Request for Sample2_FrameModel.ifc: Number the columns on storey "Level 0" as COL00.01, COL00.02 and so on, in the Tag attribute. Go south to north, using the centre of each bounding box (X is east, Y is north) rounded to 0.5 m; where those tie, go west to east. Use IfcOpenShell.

First a look at what the model holds.

```python
import ifcopenshell
import ifcopenshell.util.element
import ifcopenshell.util.placement

model = ifcopenshell.open("Sample2_FrameModel.ifc")
print(model.schema)
storey = next(s for s in model.by_type("IfcBuildingStorey") if s.Name == "Level 0")
columns = [e for e in ifcopenshell.util.element.get_decomposition(storey) if e.is_a("IfcColumn")]
for e in sorted(columns, key=lambda e: e.id()):
    origin = ifcopenshell.util.placement.get_local_placement(e.ObjectPlacement)[:3, 3]
    print(e.id(), e.Tag, e.Name, origin.round(2) + 0.0, sep=" | ")
```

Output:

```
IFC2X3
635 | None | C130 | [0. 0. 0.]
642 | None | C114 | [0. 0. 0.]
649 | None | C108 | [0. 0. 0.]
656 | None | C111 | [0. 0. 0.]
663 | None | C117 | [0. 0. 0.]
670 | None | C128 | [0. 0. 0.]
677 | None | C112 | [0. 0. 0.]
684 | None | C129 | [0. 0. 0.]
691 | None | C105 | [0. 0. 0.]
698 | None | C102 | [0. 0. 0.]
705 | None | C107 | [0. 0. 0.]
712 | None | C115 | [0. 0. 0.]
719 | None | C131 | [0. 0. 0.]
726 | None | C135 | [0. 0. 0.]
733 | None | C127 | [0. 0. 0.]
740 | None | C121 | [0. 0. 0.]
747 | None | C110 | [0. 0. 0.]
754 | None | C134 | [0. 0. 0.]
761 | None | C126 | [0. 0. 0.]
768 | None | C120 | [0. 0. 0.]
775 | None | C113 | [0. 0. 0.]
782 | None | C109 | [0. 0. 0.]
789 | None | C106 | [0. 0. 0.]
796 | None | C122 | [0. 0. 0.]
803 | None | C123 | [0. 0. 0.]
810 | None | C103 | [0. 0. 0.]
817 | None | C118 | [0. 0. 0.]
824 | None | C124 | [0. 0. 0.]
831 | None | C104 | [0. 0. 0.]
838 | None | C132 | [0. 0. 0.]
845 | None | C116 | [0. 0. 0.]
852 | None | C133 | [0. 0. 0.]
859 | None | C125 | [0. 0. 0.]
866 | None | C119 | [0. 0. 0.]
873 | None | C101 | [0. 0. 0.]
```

```python
import ifcopenshell
import ifcopenshell.geom
import ifcopenshell.util.element
import ifcopenshell.util.shape

model = ifcopenshell.open("Sample2_FrameModel.ifc")
settings = ifcopenshell.geom.settings()
settings.set("use-world-coords", True)


def centre(element):
    shape = ifcopenshell.geom.create_shape(settings, element)
    return ifcopenshell.util.shape.get_bbox_centroid(shape.geometry)


storey = next(s for s in model.by_type("IfcBuildingStorey") if s.Name == "Level 0")
columns = [e for e in ifcopenshell.util.element.get_decomposition(storey) if e.is_a("IfcColumn")]

# Insertion points can sit at a corner or the storey origin, so sort by the geometry (in metres).
centres = {e: centre(e) for e in columns}
columns.sort(key=lambda e: (round(centres[e][1] / 0.5), centres[e][0]))

for i, e in enumerate(columns, start=1):
    number = f"COL00.{i:02d}"
    e.Tag = number
    print(e.id(), number)

model.write("Sample2_FrameModel_edited.ifc")
```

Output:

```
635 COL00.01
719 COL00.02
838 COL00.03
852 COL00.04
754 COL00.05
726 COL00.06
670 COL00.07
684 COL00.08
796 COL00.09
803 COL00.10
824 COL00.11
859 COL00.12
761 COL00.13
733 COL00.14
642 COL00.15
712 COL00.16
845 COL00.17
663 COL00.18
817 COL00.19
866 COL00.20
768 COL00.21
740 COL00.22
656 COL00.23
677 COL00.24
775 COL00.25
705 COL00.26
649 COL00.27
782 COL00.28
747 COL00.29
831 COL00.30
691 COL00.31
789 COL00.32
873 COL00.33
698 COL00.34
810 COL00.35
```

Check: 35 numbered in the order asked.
